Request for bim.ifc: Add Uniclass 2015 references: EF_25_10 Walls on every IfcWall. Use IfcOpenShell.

First a look at what the model holds.

```python
import ifcopenshell

model = ifcopenshell.open("bim.ifc")
print(model.schema)
print("classifications:", [c.Name for c in model.by_type("IfcClassification")])
for ifc_class in ("IfcDoor", "IfcRoof", "IfcStair", "IfcWall", "IfcWindow"):
    print(ifc_class, len(model.by_type(ifc_class)))
```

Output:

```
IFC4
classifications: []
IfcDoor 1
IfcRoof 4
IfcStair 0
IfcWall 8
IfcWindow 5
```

```python
import ifcopenshell
import ifcopenshell.api.classification

model = ifcopenshell.open("bim.ifc")

system = ifcopenshell.api.classification.add_classification(model, classification="Uniclass 2015")

codes = {
    "IfcWall": ("EF_25_10", "Walls"),
}
for ifc_class, (code, name) in codes.items():
    products = model.by_type(ifc_class)
    ifcopenshell.api.classification.add_reference(
        model, products=products, classification=system, identification=code, name=name
    )
    print(code, len(products))

model.write("bim_updated.ifc")
```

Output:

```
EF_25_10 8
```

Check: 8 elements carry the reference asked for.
